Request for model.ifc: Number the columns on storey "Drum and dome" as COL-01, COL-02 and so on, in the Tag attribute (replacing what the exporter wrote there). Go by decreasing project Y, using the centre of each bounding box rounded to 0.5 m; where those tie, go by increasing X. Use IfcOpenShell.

First a look at what the model holds.

```python
import ifcopenshell
import ifcopenshell.util.element
import ifcopenshell.util.placement

model = ifcopenshell.open("model.ifc")
print(model.schema)
storey = next(s for s in model.by_type("IfcBuildingStorey") if s.Name == "Drum and dome")
columns = [e for e in ifcopenshell.util.element.get_decomposition(storey) if e.is_a("IfcColumn")]
for e in sorted(columns, key=lambda e: e.id()):
    origin = ifcopenshell.util.placement.get_local_placement(e.ObjectPlacement)[:3, 3]
    print(e.id(), e.Tag, e.Name, origin.round(2) + 0.0, sep=" | ")
```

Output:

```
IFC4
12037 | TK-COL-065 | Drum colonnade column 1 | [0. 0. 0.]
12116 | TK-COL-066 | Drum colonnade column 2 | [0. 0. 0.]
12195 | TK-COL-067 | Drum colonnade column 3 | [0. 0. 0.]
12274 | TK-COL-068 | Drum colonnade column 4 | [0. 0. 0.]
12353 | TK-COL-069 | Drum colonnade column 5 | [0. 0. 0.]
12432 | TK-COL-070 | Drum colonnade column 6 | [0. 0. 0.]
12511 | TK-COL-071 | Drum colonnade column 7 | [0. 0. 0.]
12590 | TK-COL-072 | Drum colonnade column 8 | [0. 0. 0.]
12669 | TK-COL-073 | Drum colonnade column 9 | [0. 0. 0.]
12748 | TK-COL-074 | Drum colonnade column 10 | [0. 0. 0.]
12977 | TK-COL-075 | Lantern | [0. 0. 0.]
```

```python
import ifcopenshell
import ifcopenshell.geom
import ifcopenshell.util.element
import ifcopenshell.util.shape

model = ifcopenshell.open("model.ifc")
settings = ifcopenshell.geom.settings()
settings.set("use-world-coords", True)


def centre(element):
    shape = ifcopenshell.geom.create_shape(settings, element)
    return ifcopenshell.util.shape.get_bbox_centroid(shape.geometry)


storey = next(s for s in model.by_type("IfcBuildingStorey") if s.Name == "Drum and dome")
columns = [e for e in ifcopenshell.util.element.get_decomposition(storey) if e.is_a("IfcColumn")]

# Insertion points can sit at a corner or the storey origin, so sort by the geometry (in metres).
centres = {e: centre(e) for e in columns}
columns.sort(key=lambda e: (-round(centres[e][1] / 0.5), centres[e][0]))

for i, e in enumerate(columns, start=1):
    number = f"COL-{i:02d}"
    e.Tag = number
    print(e.id(), number)

model.write("model_updated.ifc")
```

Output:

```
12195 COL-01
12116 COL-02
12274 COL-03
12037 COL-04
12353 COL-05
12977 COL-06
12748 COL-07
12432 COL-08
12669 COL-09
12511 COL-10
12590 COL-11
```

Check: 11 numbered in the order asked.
